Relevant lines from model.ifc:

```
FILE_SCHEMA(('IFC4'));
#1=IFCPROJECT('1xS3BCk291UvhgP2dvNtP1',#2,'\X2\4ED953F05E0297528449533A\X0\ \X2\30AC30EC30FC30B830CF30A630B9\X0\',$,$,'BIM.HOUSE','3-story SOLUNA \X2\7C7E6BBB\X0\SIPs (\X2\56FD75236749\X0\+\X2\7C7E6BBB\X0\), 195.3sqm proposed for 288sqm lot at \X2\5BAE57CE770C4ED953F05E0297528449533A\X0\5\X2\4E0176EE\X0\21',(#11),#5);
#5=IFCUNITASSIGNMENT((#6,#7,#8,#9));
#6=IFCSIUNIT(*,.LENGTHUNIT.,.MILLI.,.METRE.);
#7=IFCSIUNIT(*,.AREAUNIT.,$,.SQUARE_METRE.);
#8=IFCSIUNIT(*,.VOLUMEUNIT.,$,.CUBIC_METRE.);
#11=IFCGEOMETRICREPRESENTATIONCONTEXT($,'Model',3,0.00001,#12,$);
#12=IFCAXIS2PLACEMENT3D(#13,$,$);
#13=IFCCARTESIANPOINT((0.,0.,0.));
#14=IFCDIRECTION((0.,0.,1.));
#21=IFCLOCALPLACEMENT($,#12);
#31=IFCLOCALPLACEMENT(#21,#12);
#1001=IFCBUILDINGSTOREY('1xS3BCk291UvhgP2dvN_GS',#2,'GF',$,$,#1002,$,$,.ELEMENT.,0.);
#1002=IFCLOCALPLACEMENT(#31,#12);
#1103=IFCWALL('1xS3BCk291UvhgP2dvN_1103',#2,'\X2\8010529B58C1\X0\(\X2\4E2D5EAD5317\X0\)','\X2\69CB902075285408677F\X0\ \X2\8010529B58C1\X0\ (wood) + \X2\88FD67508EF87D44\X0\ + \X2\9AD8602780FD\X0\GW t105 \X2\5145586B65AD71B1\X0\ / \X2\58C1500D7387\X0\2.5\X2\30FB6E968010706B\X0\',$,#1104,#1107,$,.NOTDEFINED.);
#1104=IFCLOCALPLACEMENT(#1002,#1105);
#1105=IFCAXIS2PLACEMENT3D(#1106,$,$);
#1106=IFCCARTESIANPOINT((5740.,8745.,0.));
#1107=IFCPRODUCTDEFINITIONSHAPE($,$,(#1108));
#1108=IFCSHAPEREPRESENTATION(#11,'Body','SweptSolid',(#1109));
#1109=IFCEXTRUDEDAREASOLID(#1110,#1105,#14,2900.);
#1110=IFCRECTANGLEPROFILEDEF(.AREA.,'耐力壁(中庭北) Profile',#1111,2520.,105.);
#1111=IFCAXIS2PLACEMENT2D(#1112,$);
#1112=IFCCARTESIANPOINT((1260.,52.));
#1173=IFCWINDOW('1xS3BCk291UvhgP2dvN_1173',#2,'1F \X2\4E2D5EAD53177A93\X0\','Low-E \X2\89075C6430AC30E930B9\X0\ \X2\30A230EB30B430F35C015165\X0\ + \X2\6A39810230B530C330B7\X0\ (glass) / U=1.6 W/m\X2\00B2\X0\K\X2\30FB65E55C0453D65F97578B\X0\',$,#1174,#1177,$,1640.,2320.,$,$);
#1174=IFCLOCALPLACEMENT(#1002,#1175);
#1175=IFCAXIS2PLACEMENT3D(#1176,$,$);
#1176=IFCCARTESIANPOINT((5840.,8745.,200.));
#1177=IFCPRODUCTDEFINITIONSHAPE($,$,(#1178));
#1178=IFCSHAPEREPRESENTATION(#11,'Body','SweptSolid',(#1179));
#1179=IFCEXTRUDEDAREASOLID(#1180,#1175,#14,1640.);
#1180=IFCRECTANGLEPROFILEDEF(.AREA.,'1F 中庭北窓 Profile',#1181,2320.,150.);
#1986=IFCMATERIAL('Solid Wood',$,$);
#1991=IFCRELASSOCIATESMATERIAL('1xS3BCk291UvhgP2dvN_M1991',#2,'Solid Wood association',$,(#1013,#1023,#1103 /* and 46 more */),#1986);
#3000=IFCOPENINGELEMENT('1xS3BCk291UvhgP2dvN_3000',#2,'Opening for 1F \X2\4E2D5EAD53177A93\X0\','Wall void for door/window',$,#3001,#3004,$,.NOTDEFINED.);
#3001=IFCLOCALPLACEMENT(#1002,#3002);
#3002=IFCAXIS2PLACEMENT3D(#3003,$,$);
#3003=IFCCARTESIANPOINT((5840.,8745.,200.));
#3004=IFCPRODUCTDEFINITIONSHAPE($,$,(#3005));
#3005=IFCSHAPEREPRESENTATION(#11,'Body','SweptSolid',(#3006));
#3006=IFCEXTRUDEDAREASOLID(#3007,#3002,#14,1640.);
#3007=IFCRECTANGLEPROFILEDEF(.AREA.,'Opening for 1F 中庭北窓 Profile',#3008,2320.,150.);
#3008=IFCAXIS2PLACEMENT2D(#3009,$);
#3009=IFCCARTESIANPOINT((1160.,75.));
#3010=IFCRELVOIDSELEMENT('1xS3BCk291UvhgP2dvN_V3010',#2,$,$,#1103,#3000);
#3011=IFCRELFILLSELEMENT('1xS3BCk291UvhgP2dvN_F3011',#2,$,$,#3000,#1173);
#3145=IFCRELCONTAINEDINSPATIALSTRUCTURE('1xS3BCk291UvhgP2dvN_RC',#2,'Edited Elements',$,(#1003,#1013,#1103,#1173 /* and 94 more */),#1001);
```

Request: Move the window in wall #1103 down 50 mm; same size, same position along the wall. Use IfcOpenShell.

```python
import numpy as np
import ifcopenshell
import ifcopenshell.api.geometry
import ifcopenshell.util.placement
import ifcopenshell.util.unit

model = ifcopenshell.open("model.ifc")
unit_scale = ifcopenshell.util.unit.calculate_unit_scale(model)

window = model.by_id(1173)
opening = window.FillsVoids[0].RelatingOpeningElement
dz = -50.0

shift = np.array([0.0, 0.0, dz])
# The window is not placed relative to its opening, so move both.
for product in (opening, window):
    matrix = ifcopenshell.util.placement.get_local_placement(product.ObjectPlacement)
    matrix[:3, 3] += shift
    ifcopenshell.api.geometry.edit_object_placement(model, product=product, matrix=matrix, is_si=False)

print(f"moved by {dz * unit_scale:+.3f} m")

model.write("model_rev.ifc")
```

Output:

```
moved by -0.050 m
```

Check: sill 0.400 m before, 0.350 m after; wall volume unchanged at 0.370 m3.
